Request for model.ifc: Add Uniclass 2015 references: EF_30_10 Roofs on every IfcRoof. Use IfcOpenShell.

First a look at what the model holds.

```python
import ifcopenshell

model = ifcopenshell.open("model.ifc")
print(model.schema)
print("classifications:", [c.Name for c in model.by_type("IfcClassification")])
for ifc_class in ("IfcDoor", "IfcRoof", "IfcStair", "IfcWall", "IfcWindow"):
    print(ifc_class, len(model.by_type(ifc_class)))
```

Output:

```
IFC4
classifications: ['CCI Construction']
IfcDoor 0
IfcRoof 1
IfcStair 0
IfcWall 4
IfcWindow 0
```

```python
import ifcopenshell
import ifcopenshell.api.classification

model = ifcopenshell.open("model.ifc")

system = ifcopenshell.api.classification.add_classification(model, classification="Uniclass 2015")

codes = {
    "IfcRoof": ("EF_30_10", "Roofs"),
}
for ifc_class, (code, name) in codes.items():
    products = model.by_type(ifc_class)
    ifcopenshell.api.classification.add_reference(
        model, products=products, classification=system, identification=code, name=name
    )
    print(code, len(products))

model.write("model_v2.ifc")
```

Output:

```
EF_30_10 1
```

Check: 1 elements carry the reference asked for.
